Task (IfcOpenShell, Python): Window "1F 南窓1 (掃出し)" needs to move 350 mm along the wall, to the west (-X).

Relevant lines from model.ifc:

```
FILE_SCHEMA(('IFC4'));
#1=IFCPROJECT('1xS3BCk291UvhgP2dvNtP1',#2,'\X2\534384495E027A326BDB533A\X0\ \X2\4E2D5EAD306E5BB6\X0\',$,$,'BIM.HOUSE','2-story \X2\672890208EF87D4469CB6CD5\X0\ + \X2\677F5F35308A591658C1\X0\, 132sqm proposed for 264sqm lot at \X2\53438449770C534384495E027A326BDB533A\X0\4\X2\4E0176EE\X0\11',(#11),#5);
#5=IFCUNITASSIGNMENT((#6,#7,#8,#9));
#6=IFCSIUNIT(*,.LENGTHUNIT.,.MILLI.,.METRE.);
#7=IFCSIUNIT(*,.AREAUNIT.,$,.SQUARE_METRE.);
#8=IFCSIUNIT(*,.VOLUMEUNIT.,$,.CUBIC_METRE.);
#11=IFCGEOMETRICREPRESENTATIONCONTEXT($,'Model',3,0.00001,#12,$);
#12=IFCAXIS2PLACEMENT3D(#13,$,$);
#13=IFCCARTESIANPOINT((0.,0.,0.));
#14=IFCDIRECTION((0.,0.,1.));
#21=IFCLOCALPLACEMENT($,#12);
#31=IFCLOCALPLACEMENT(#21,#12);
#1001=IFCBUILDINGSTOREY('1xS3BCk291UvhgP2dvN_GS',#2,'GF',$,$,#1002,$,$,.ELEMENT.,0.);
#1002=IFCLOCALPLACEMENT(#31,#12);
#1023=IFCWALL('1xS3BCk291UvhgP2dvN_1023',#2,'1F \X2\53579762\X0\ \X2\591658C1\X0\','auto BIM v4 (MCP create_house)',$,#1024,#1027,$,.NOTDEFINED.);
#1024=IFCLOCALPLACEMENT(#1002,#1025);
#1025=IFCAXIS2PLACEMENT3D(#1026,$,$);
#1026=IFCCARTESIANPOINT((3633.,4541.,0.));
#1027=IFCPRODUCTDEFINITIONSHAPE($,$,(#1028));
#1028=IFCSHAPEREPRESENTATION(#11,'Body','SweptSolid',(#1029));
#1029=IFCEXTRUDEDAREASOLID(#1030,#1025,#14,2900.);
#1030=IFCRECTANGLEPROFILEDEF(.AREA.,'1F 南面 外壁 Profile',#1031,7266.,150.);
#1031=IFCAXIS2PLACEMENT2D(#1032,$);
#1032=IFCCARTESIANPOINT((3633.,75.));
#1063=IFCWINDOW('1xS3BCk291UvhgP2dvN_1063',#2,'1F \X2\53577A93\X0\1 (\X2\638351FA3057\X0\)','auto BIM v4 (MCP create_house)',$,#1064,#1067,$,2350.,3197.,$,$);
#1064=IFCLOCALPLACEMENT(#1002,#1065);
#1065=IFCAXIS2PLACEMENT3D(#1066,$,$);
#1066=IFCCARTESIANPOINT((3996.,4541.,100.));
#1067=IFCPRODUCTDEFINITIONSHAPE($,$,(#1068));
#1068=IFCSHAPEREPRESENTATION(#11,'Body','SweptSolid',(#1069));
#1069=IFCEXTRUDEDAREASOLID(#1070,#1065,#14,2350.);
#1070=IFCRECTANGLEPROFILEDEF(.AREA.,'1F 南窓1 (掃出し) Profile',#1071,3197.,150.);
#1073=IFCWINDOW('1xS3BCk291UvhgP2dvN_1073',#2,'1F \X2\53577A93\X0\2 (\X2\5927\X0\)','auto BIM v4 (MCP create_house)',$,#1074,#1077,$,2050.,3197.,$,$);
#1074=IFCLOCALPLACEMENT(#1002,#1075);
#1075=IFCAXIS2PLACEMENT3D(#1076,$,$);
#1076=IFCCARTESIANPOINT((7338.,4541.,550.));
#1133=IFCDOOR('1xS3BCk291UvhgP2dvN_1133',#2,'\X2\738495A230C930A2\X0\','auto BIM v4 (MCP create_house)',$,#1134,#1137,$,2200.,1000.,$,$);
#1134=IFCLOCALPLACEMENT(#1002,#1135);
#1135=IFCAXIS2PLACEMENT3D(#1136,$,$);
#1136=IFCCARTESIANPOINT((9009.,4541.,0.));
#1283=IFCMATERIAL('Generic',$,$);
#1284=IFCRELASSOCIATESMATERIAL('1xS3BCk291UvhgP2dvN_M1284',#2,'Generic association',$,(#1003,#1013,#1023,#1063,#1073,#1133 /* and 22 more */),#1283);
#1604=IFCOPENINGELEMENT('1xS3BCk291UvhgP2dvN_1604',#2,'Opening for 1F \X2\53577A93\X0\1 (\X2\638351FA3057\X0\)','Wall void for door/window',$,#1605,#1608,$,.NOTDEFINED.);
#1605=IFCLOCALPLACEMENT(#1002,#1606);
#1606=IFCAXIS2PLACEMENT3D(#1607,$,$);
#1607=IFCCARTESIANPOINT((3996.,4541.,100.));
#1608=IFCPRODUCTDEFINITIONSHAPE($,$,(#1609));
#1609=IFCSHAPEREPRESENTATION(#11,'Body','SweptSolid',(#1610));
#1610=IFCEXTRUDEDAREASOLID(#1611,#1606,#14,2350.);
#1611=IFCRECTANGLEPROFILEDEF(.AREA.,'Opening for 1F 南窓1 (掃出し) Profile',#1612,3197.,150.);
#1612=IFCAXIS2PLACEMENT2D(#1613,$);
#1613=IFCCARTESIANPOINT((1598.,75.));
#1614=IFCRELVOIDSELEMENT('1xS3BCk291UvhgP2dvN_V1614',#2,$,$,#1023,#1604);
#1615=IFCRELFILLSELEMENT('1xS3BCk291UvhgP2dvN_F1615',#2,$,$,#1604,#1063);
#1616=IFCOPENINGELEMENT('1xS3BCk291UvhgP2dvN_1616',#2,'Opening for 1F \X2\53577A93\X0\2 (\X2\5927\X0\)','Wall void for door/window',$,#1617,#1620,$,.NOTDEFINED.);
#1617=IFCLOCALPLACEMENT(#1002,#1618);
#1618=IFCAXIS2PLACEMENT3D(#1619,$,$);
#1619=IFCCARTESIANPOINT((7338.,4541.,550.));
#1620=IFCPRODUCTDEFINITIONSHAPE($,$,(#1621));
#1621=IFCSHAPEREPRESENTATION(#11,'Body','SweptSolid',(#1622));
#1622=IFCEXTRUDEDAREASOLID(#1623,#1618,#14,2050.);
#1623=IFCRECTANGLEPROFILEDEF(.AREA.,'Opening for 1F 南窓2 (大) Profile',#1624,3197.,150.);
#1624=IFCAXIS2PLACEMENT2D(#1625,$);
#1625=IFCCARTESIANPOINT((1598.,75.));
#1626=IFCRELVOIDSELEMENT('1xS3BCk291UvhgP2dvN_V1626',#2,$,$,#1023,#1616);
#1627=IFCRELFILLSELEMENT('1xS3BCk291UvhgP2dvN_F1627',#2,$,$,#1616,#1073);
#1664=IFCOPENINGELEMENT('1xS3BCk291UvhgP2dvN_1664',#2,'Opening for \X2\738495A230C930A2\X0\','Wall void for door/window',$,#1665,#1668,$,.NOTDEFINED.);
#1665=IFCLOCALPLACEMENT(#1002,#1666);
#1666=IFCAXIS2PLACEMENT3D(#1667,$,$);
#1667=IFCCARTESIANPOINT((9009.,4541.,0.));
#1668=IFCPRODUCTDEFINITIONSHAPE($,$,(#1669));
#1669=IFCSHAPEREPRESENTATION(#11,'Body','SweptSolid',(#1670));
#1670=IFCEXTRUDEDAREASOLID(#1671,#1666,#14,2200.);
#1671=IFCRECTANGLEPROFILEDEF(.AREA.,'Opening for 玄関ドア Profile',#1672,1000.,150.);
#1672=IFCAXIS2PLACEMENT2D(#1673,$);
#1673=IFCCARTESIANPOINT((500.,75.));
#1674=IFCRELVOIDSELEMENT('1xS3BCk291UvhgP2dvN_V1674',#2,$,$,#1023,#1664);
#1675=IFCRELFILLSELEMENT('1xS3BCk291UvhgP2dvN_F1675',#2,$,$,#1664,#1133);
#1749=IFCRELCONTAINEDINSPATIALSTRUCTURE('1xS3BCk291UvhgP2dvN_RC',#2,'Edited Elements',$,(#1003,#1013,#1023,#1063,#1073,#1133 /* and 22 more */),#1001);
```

```python
import ifcopenshell
import ifcopenshell.api.geometry
import ifcopenshell.util.placement

model = ifcopenshell.open("model.ifc")

window = model.by_guid("1xS3BCk291UvhgP2dvN_1063")
opening = window.FillsVoids[0].RelatingOpeningElement
wall = opening.VoidsElements[0].RelatingBuildingElement

wall_matrix = ifcopenshell.util.placement.get_local_placement(wall.ObjectPlacement)
shift = wall_matrix[:3, 0] * -350.0
before = ifcopenshell.util.placement.get_local_placement(window.ObjectPlacement)[:3, 3].copy()

# The window is not placed relative to its opening, so move both.
for product in (opening, window):
    matrix = ifcopenshell.util.placement.get_local_placement(product.ObjectPlacement)
    matrix[:3, 3] += shift
    ifcopenshell.api.geometry.edit_object_placement(model, product=product, matrix=matrix, is_si=False)

after = ifcopenshell.util.placement.get_local_placement(window.ObjectPlacement)[:3, 3]
print("window moved by", (after - before).round(3) + 0.0)

model.write("model-out.ifc")
```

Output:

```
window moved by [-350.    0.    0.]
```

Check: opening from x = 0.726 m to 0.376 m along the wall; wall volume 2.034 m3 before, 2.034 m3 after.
